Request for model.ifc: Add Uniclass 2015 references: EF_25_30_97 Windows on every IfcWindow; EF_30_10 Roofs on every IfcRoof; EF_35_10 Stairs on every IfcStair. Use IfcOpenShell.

First a look at what the model holds.

```python
import ifcopenshell

model = ifcopenshell.open("model.ifc")
print(model.schema)
print("classifications:", [c.Name for c in model.by_type("IfcClassification")])
for ifc_class in ("IfcDoor", "IfcRoof", "IfcStair", "IfcWall", "IfcWindow"):
    print(ifc_class, len(model.by_type(ifc_class)))
```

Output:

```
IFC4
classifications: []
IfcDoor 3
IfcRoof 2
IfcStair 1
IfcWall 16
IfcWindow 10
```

```python
import ifcopenshell
import ifcopenshell.api.classification

model = ifcopenshell.open("model.ifc")

system = ifcopenshell.api.classification.add_classification(model, classification="Uniclass 2015")

codes = {
    "IfcWindow": ("EF_25_30_97", "Windows"),
    "IfcRoof": ("EF_30_10", "Roofs"),
    "IfcStair": ("EF_35_10", "Stairs"),
}
for ifc_class, (code, name) in codes.items():
    products = model.by_type(ifc_class)
    ifcopenshell.api.classification.add_reference(
        model, products=products, classification=system, identification=code, name=name
    )
    print(code, len(products))

model.write("model_v2.ifc")
```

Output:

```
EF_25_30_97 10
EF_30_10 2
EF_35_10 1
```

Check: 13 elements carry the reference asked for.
